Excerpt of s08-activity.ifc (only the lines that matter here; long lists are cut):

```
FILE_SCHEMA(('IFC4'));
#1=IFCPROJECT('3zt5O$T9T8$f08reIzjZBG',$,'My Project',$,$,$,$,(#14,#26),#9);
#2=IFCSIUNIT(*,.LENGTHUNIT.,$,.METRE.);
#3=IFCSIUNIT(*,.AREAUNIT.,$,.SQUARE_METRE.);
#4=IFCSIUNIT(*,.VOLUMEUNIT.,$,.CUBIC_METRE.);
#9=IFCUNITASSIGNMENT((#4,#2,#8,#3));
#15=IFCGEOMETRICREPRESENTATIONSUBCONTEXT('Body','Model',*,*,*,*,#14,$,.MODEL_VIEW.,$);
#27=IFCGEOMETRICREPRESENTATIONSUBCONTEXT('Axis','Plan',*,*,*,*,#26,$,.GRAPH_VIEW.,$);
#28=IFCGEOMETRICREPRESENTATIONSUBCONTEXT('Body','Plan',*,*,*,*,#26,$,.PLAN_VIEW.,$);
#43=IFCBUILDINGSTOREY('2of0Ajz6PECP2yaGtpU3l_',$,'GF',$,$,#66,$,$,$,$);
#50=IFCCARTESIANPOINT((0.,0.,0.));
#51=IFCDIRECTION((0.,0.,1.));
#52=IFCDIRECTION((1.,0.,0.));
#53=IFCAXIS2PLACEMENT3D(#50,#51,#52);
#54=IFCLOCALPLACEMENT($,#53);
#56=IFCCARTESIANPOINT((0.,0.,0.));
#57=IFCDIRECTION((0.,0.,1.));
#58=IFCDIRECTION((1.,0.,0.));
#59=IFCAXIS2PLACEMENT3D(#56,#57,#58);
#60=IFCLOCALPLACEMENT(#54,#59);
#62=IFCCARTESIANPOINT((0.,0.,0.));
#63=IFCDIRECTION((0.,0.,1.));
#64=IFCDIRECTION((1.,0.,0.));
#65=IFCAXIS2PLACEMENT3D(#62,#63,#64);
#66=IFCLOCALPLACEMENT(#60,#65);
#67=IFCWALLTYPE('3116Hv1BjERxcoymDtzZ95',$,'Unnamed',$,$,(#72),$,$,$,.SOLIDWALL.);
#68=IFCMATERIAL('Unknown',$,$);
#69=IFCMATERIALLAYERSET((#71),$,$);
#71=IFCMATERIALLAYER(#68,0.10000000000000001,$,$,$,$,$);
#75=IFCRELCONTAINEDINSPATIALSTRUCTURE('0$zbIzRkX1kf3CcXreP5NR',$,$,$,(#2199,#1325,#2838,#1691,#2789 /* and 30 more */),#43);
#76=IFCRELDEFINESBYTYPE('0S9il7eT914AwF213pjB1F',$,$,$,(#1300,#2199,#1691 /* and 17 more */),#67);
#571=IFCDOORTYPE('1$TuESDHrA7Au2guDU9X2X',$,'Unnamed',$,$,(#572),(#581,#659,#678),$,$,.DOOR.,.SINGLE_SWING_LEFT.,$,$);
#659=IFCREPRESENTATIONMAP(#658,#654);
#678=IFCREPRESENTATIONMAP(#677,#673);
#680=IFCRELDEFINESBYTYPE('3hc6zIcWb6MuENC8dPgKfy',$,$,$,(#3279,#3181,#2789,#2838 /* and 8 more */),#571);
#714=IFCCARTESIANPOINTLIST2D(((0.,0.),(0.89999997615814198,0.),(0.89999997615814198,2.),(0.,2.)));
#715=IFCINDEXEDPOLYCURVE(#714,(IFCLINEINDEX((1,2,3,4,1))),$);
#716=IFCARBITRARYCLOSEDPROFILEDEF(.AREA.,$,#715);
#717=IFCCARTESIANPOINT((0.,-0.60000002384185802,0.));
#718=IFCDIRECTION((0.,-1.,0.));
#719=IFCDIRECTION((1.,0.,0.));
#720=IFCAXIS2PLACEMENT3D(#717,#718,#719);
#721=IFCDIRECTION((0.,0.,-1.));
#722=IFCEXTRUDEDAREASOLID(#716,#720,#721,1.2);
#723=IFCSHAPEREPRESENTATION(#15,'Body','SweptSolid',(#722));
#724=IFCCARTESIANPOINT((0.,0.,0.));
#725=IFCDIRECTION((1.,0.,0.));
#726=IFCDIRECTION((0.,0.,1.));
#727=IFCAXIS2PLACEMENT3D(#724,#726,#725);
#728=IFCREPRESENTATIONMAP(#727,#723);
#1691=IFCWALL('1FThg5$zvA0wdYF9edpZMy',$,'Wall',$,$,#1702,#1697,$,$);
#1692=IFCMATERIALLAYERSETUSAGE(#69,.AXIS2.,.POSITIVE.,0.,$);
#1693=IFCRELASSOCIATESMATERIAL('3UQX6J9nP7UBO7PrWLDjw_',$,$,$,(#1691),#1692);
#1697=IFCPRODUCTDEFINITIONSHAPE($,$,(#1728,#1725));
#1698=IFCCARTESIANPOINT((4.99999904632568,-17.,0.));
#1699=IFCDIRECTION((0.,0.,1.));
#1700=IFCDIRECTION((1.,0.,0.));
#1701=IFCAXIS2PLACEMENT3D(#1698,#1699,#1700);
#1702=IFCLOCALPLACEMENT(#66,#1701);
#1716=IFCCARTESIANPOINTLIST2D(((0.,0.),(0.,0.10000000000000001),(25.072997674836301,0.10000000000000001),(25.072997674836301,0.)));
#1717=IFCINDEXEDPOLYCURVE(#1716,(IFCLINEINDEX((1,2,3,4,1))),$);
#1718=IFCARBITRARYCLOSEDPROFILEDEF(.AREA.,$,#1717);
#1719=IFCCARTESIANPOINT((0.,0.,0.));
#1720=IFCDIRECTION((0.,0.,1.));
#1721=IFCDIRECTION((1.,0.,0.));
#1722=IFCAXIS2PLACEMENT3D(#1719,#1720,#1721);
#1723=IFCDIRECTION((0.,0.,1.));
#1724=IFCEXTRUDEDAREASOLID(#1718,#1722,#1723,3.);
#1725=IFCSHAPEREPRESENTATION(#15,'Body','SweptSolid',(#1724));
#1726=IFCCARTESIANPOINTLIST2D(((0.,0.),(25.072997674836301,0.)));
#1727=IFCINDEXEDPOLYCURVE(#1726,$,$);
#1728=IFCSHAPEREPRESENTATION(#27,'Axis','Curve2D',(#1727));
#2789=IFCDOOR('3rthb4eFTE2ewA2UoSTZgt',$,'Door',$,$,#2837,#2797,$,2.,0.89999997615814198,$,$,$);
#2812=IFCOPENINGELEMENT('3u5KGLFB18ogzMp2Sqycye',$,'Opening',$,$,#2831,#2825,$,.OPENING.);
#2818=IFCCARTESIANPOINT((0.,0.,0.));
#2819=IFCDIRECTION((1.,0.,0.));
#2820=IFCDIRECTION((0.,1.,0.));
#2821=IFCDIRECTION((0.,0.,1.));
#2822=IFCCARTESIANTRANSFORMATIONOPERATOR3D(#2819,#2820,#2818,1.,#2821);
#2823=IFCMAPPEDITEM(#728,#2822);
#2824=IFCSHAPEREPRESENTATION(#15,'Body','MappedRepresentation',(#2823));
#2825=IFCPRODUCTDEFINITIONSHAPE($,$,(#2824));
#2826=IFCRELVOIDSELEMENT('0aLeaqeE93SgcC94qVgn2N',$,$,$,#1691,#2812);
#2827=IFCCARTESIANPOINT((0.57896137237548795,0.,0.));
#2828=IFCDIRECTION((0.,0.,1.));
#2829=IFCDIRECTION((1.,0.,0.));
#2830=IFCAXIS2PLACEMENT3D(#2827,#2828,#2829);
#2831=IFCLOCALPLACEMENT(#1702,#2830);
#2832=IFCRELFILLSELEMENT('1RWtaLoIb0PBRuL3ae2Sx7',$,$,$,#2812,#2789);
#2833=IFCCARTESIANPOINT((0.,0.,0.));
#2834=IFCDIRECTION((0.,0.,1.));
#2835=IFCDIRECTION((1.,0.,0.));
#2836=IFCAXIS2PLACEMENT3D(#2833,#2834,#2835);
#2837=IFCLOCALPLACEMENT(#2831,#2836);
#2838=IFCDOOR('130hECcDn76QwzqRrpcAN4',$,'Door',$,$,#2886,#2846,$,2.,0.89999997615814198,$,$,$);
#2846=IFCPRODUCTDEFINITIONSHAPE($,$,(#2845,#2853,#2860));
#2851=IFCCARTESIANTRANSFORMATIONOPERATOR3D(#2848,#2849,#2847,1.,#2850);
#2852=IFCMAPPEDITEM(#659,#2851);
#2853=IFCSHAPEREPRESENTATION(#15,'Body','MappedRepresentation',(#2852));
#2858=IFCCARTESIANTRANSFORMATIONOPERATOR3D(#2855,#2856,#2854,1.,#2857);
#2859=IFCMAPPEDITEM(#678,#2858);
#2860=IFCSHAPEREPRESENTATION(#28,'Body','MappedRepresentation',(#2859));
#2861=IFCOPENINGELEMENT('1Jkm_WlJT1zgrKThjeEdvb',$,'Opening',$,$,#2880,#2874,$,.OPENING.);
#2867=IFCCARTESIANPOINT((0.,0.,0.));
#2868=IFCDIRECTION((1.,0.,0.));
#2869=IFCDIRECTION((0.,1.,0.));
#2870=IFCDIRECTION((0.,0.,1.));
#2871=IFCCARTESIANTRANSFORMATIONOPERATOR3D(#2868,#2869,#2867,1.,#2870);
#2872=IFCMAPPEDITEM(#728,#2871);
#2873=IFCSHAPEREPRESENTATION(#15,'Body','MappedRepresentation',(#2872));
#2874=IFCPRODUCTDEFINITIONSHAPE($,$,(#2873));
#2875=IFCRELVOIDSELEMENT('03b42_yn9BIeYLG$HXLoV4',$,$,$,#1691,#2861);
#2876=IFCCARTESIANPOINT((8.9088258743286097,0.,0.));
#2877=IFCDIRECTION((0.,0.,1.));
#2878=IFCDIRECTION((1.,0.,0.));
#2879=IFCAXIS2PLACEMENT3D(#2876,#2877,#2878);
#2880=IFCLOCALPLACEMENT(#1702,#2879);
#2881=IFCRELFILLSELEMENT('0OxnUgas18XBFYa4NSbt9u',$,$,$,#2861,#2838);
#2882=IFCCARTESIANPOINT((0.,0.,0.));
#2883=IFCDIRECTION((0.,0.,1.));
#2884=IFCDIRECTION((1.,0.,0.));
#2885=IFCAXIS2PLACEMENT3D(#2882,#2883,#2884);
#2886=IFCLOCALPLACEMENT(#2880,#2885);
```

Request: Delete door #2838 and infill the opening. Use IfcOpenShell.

```python
import ifcopenshell
import ifcopenshell.api.feature
import ifcopenshell.api.root
import ifcopenshell.geom
import ifcopenshell.util.shape

model = ifcopenshell.open("s08-activity.ifc")
settings = ifcopenshell.geom.settings()


def volume(element):
    """Net volume in cubic metres, openings subtracted."""
    shape = ifcopenshell.geom.create_shape(settings, element)
    return ifcopenshell.util.shape.get_volume(shape.geometry)


door = model.by_guid("130hECcDn76QwzqRrpcAN4")
opening = door.FillsVoids[0].RelatingOpeningElement
wall = opening.VoidsElements[0].RelatingBuildingElement
before = volume(wall)

ifcopenshell.api.root.remove_product(model, product=door)
ifcopenshell.api.feature.remove_feature(model, feature=opening)

after = volume(wall)

print(f"wall volume {before:.3f} -> {after:.3f} m3")

model.write("s08-activity_v2.ifc")
```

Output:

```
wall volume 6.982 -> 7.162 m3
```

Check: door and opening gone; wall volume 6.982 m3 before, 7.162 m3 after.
